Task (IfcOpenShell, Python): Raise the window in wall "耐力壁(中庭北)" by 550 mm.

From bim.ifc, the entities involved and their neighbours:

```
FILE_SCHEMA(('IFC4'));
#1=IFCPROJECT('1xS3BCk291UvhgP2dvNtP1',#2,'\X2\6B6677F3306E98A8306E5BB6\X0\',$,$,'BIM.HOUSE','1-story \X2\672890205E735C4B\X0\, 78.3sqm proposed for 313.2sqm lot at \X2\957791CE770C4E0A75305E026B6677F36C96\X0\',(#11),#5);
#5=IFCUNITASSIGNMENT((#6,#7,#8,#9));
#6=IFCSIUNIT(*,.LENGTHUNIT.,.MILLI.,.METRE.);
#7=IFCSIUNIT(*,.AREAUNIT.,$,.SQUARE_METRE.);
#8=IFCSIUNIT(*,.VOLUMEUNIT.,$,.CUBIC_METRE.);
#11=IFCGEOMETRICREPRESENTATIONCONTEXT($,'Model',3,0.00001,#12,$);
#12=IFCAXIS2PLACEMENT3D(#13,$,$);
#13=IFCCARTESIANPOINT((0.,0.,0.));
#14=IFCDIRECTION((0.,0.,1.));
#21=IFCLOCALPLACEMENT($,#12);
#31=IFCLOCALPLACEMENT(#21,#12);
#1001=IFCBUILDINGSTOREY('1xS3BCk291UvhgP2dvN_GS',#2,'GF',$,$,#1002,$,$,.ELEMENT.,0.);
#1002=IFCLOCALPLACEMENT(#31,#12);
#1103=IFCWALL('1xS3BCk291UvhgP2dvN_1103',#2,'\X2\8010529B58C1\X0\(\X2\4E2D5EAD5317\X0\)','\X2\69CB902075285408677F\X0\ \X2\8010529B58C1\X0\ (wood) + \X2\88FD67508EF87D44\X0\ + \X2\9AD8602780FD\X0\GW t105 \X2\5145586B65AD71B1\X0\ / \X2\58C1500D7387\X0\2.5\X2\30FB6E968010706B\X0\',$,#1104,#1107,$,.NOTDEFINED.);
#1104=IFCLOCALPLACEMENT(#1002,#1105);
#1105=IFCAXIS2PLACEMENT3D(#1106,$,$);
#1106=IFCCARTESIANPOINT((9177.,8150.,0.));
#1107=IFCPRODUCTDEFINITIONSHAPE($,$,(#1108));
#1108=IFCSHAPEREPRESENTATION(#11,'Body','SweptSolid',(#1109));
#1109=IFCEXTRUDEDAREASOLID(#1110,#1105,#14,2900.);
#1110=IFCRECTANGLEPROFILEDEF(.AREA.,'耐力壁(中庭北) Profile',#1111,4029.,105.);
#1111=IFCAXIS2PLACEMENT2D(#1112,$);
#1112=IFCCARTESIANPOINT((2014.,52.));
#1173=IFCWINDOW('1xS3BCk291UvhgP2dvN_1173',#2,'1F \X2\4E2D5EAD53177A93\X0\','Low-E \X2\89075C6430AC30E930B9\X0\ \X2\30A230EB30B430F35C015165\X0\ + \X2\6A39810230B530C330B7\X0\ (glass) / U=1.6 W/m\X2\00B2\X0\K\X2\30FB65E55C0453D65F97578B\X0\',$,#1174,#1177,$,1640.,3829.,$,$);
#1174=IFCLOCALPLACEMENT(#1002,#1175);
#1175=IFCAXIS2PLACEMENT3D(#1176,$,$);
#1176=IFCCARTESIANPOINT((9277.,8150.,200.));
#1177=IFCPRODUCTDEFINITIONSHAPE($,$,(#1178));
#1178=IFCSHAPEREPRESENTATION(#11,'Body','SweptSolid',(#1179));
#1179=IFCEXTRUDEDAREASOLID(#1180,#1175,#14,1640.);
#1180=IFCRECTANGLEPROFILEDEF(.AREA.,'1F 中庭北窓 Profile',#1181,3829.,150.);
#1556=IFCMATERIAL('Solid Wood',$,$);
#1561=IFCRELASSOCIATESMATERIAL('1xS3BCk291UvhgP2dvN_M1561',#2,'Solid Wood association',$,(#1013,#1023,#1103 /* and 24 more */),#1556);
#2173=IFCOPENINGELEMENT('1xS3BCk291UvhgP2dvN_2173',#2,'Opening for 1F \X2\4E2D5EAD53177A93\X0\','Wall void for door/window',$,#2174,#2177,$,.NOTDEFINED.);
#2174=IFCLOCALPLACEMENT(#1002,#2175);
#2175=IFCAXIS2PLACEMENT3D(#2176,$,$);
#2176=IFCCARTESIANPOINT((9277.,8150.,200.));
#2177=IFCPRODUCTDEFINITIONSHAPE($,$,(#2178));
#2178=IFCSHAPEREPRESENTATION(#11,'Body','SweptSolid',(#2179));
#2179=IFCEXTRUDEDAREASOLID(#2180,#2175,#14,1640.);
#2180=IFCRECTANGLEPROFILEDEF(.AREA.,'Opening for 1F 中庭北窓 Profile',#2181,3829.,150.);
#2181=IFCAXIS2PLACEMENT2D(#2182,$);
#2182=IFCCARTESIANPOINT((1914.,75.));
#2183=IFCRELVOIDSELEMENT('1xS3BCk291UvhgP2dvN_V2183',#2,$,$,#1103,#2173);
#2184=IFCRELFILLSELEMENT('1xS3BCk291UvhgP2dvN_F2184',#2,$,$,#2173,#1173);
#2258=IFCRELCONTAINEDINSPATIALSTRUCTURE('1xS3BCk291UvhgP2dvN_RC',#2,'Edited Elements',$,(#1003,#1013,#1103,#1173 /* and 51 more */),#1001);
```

```python
import numpy as np
import ifcopenshell
import ifcopenshell.api.geometry
import ifcopenshell.util.placement
import ifcopenshell.util.unit

model = ifcopenshell.open("bim.ifc")
unit_scale = ifcopenshell.util.unit.calculate_unit_scale(model)

window = model.by_guid("1xS3BCk291UvhgP2dvN_1173")
opening = window.FillsVoids[0].RelatingOpeningElement
dz = 0.55 / unit_scale

shift = np.array([0.0, 0.0, dz])
# The window is not placed relative to its opening, so move both.
for product in (opening, window):
    matrix = ifcopenshell.util.placement.get_local_placement(product.ObjectPlacement)
    matrix[:3, 3] += shift
    ifcopenshell.api.geometry.edit_object_placement(model, product=product, matrix=matrix, is_si=False)

print(f"moved by {dz * unit_scale:+.3f} m")

model.write("bim-out.ifc")
```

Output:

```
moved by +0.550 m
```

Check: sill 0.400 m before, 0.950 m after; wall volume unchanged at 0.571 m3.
